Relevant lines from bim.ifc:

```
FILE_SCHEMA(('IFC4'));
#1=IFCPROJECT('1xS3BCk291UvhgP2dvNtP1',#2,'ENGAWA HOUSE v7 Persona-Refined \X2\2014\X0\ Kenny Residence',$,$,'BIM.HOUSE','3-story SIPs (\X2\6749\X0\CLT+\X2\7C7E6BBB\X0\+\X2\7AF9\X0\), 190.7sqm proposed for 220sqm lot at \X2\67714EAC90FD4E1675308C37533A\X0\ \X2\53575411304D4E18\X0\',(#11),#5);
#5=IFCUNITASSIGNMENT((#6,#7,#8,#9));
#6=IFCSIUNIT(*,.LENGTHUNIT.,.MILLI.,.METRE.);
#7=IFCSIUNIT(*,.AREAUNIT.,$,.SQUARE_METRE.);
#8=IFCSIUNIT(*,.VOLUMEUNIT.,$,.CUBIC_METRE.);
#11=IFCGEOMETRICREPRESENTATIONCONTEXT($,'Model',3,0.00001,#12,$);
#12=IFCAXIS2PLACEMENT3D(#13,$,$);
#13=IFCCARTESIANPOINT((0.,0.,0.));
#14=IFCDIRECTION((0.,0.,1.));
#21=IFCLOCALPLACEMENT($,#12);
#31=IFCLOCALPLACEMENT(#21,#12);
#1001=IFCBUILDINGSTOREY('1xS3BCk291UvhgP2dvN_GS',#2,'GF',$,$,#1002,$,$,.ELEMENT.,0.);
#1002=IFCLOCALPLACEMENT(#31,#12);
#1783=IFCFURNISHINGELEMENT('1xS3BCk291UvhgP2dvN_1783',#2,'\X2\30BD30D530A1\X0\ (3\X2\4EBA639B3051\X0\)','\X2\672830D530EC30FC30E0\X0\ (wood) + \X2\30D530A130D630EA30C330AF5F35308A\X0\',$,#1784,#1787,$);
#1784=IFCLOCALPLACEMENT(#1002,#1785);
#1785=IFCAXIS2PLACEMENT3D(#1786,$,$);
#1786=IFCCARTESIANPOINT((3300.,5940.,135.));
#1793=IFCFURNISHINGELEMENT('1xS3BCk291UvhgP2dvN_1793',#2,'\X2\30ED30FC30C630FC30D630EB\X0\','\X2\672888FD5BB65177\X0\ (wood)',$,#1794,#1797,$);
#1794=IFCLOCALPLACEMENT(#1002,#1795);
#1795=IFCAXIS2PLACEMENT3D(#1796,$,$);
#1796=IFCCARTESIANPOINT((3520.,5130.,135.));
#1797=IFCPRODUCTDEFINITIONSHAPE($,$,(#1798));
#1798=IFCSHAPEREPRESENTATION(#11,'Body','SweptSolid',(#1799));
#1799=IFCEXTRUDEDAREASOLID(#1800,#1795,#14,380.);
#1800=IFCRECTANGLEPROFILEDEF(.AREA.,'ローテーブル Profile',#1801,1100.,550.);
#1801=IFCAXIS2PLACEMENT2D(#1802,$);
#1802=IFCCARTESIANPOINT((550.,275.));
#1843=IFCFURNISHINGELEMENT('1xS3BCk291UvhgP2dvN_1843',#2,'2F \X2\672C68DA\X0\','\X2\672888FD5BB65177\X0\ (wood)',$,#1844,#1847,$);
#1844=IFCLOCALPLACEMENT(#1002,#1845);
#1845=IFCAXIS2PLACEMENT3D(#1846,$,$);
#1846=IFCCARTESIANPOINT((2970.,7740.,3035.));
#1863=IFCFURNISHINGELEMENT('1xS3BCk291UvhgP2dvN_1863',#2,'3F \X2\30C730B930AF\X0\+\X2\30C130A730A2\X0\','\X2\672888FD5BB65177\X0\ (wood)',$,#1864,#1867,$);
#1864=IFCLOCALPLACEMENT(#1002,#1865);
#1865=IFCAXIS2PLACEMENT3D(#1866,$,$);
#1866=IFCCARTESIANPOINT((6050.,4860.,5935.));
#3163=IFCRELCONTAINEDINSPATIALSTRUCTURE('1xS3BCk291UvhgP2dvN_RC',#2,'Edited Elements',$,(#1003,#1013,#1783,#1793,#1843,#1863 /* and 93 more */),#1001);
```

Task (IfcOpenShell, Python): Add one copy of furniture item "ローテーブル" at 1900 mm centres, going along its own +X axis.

```python
import ifcopenshell
import ifcopenshell.api.geometry
import ifcopenshell.api.root
import ifcopenshell.util.element
import ifcopenshell.util.placement

model = ifcopenshell.open("bim.ifc")


def reuse_history(source, copy):
    """copy_class also copies each property set's owner history, people and application; keep the originals."""
    for rel in copy.IsDefinedBy:
        if rel.is_a("IfcRelDefinesByProperties") and (history := rel.RelatingPropertyDefinition.OwnerHistory):
            rel.RelatingPropertyDefinition.OwnerHistory = source.OwnerHistory
            ifcopenshell.util.element.remove_deep2(model, history)


source = model.by_guid("1xS3BCk291UvhgP2dvN_1793")
base = ifcopenshell.util.placement.get_local_placement(source.ObjectPlacement)
step = base[:3, 0] * 1900.0

for i in range(1, 2):
    copy = ifcopenshell.api.root.copy_class(model, product=source)
    copy.Representation = ifcopenshell.util.element.copy_deep(
        model, source.Representation, exclude=["IfcGeometricRepresentationContext", "IfcRepresentationMap"]
    )
    reuse_history(source, copy)
    matrix = base.copy()
    matrix[:3, 3] += i * step
    print("added at", matrix[:3, 3].round(3) + 0.0)
    ifcopenshell.api.geometry.edit_object_placement(model, product=copy, matrix=matrix, is_si=False)

model.write("bim_edited.ifc")
```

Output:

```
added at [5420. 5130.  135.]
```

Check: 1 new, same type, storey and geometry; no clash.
